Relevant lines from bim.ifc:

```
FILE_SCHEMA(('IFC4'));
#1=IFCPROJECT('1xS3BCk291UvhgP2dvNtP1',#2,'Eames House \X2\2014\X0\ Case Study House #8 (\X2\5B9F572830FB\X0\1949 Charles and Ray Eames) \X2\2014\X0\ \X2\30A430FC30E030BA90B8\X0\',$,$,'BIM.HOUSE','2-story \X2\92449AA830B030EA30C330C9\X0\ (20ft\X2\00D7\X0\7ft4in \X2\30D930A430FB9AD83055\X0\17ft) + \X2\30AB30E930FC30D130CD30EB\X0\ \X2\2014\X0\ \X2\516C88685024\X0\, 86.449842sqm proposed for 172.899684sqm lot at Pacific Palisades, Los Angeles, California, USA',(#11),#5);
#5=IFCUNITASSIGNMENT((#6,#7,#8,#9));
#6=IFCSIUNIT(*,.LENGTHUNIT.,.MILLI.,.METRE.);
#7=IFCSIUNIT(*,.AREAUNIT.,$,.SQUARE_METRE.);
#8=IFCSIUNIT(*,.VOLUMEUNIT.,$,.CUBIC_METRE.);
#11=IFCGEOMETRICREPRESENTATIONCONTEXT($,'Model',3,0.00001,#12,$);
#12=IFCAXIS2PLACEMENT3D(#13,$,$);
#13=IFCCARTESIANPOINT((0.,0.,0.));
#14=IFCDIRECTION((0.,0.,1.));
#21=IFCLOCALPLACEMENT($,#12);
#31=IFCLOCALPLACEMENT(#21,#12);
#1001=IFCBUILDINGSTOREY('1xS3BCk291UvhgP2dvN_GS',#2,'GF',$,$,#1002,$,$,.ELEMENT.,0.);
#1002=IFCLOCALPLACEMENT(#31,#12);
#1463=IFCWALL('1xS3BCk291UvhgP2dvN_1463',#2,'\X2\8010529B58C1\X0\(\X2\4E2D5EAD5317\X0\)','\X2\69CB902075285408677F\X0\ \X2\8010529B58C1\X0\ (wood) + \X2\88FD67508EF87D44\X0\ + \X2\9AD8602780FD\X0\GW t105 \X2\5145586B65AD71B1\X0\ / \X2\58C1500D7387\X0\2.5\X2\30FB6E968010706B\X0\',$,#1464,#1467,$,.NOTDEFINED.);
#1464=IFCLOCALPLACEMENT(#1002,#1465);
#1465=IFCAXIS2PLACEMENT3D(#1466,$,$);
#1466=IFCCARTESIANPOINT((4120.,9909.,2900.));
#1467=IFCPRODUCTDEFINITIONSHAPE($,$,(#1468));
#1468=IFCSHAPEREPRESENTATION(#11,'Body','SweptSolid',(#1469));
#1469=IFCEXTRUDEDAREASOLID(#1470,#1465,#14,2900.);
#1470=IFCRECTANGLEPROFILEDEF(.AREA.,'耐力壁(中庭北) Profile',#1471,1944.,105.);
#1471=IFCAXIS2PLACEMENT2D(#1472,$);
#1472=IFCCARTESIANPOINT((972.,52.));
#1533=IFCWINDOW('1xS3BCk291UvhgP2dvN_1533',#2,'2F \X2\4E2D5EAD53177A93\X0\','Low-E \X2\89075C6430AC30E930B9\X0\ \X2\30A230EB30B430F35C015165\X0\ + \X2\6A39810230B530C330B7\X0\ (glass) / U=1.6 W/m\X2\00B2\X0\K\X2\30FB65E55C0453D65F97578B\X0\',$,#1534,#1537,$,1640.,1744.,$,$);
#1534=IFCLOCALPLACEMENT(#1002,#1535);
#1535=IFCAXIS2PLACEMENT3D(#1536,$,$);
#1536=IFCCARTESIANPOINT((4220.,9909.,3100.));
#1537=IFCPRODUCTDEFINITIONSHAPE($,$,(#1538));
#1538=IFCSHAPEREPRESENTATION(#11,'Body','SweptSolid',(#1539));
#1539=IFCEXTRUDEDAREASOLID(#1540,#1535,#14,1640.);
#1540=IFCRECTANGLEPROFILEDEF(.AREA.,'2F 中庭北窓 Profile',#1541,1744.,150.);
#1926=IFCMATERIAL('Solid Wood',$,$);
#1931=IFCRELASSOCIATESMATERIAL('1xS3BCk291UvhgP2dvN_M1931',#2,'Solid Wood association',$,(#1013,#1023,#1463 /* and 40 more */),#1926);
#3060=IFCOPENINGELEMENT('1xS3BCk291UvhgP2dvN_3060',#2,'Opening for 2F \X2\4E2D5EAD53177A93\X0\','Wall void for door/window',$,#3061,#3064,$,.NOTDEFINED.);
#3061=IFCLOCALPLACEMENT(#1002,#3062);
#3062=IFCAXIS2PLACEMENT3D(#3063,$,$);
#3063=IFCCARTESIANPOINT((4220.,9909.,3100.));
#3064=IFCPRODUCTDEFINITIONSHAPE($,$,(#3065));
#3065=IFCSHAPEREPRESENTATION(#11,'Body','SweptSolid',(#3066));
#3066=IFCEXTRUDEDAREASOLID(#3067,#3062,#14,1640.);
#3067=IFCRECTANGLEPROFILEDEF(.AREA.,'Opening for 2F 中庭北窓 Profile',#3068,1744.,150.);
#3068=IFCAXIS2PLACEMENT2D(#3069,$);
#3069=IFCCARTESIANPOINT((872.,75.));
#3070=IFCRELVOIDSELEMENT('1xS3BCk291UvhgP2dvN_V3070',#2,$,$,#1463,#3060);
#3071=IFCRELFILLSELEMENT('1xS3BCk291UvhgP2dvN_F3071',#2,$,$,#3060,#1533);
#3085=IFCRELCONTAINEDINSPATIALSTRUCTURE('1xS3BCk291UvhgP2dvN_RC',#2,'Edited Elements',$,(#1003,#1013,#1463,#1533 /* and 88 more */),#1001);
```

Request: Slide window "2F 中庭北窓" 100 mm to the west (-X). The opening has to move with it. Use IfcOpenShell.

```python
import ifcopenshell
import ifcopenshell.api.geometry
import ifcopenshell.util.placement

model = ifcopenshell.open("bim.ifc")

window = model.by_id(1533)
opening = window.FillsVoids[0].RelatingOpeningElement
wall = opening.VoidsElements[0].RelatingBuildingElement

wall_matrix = ifcopenshell.util.placement.get_local_placement(wall.ObjectPlacement)
shift = wall_matrix[:3, 0] * -100.0
before = ifcopenshell.util.placement.get_local_placement(window.ObjectPlacement)[:3, 3].copy()

# The window is not placed relative to its opening, so move both.
for product in (opening, window):
    matrix = ifcopenshell.util.placement.get_local_placement(product.ObjectPlacement)
    matrix[:3, 3] += shift
    ifcopenshell.api.geometry.edit_object_placement(model, product=product, matrix=matrix, is_si=False)

after = ifcopenshell.util.placement.get_local_placement(window.ObjectPlacement)[:3, 3]
print("window moved by", (after - before).round(3) + 0.0)

model.write("bim_updated.ifc")
```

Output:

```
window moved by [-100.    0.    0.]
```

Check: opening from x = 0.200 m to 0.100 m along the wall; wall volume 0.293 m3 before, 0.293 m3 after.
